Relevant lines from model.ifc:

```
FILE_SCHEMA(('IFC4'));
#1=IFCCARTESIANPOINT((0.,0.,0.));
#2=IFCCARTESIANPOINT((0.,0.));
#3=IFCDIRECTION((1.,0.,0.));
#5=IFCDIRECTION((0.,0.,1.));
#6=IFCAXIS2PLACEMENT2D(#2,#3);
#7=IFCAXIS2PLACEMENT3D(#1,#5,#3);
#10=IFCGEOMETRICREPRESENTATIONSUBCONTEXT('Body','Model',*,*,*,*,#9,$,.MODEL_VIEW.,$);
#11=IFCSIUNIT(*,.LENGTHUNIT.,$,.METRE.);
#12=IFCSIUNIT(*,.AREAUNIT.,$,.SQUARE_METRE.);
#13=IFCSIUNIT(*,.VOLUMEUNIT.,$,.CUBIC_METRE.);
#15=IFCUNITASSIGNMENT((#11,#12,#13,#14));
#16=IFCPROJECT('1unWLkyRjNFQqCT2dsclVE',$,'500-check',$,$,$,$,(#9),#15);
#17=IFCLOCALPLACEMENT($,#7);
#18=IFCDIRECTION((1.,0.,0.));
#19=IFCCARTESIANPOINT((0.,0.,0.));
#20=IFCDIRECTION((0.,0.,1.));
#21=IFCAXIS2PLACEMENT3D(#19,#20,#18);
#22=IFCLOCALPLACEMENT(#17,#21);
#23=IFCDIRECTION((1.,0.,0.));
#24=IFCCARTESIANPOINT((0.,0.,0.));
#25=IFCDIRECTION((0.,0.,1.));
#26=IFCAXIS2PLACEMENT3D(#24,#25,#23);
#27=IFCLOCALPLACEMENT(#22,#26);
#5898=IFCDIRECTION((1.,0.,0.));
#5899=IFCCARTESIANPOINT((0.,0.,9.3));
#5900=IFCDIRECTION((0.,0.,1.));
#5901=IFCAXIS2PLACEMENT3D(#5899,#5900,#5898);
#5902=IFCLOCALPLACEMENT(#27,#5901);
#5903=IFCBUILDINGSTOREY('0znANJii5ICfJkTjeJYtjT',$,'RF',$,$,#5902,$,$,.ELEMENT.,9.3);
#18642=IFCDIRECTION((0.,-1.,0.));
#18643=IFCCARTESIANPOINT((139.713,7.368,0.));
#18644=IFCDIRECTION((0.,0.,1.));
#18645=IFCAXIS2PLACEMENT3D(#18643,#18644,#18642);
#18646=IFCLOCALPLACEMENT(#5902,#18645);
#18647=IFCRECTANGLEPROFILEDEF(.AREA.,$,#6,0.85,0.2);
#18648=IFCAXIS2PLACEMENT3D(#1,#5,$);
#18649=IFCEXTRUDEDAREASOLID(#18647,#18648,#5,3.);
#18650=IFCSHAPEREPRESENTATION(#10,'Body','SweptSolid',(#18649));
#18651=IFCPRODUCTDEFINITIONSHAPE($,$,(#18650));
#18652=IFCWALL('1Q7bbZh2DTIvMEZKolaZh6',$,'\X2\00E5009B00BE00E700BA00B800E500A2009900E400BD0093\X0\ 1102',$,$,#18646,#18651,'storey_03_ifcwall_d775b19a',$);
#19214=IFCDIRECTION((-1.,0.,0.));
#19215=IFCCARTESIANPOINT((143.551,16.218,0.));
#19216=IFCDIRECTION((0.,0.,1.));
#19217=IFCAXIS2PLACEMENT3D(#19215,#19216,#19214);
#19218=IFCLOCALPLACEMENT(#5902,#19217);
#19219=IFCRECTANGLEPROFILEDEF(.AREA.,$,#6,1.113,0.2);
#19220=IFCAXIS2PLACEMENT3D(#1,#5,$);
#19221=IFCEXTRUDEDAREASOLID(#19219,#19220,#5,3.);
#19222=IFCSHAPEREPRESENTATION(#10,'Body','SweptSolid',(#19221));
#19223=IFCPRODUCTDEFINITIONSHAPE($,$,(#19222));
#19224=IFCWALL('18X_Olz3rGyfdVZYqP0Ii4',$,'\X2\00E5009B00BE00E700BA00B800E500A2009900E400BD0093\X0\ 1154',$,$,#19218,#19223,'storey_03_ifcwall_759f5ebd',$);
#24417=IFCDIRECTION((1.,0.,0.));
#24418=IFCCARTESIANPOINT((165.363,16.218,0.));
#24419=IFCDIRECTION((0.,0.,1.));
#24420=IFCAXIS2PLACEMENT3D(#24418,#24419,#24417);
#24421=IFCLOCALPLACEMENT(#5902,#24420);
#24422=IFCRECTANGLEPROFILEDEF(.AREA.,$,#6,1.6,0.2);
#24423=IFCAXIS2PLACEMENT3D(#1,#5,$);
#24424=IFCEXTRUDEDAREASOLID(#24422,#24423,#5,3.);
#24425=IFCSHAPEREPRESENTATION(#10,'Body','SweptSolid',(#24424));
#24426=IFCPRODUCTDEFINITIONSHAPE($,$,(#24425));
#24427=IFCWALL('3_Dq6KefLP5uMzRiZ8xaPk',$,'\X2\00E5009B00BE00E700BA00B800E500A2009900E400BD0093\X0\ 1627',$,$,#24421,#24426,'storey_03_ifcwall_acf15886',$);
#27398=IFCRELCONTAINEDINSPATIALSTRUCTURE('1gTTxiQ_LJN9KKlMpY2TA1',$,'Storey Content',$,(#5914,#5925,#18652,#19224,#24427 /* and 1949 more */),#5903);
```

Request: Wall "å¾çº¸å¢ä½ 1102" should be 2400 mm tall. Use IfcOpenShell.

```python
import ifcopenshell
import ifcopenshell.geom
import ifcopenshell.util.representation
import ifcopenshell.util.shape
import ifcopenshell.util.unit

model = ifcopenshell.open("model.ifc")
unit_scale = ifcopenshell.util.unit.calculate_unit_scale(model)
settings = ifcopenshell.geom.settings()


def volume(element):
    """Net volume in cubic metres, openings subtracted."""
    shape = ifcopenshell.geom.create_shape(settings, element)
    return ifcopenshell.util.shape.get_volume(shape.geometry)


wall = model.by_guid("1Q7bbZh2DTIvMEZKolaZh6")
before = volume(wall)

body = ifcopenshell.util.representation.get_representation(wall, "Model", "Body")
solid = body.Items[0]
old_height = solid.Depth
solid.Depth = 2.4 / unit_scale
after = volume(wall)

print(f"height {old_height:g} -> {solid.Depth:g}, volume {before:.3f} -> {after:.3f} m3")

model.write("model-out.ifc")
```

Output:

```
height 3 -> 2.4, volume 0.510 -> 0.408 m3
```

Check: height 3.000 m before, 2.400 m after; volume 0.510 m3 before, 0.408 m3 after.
